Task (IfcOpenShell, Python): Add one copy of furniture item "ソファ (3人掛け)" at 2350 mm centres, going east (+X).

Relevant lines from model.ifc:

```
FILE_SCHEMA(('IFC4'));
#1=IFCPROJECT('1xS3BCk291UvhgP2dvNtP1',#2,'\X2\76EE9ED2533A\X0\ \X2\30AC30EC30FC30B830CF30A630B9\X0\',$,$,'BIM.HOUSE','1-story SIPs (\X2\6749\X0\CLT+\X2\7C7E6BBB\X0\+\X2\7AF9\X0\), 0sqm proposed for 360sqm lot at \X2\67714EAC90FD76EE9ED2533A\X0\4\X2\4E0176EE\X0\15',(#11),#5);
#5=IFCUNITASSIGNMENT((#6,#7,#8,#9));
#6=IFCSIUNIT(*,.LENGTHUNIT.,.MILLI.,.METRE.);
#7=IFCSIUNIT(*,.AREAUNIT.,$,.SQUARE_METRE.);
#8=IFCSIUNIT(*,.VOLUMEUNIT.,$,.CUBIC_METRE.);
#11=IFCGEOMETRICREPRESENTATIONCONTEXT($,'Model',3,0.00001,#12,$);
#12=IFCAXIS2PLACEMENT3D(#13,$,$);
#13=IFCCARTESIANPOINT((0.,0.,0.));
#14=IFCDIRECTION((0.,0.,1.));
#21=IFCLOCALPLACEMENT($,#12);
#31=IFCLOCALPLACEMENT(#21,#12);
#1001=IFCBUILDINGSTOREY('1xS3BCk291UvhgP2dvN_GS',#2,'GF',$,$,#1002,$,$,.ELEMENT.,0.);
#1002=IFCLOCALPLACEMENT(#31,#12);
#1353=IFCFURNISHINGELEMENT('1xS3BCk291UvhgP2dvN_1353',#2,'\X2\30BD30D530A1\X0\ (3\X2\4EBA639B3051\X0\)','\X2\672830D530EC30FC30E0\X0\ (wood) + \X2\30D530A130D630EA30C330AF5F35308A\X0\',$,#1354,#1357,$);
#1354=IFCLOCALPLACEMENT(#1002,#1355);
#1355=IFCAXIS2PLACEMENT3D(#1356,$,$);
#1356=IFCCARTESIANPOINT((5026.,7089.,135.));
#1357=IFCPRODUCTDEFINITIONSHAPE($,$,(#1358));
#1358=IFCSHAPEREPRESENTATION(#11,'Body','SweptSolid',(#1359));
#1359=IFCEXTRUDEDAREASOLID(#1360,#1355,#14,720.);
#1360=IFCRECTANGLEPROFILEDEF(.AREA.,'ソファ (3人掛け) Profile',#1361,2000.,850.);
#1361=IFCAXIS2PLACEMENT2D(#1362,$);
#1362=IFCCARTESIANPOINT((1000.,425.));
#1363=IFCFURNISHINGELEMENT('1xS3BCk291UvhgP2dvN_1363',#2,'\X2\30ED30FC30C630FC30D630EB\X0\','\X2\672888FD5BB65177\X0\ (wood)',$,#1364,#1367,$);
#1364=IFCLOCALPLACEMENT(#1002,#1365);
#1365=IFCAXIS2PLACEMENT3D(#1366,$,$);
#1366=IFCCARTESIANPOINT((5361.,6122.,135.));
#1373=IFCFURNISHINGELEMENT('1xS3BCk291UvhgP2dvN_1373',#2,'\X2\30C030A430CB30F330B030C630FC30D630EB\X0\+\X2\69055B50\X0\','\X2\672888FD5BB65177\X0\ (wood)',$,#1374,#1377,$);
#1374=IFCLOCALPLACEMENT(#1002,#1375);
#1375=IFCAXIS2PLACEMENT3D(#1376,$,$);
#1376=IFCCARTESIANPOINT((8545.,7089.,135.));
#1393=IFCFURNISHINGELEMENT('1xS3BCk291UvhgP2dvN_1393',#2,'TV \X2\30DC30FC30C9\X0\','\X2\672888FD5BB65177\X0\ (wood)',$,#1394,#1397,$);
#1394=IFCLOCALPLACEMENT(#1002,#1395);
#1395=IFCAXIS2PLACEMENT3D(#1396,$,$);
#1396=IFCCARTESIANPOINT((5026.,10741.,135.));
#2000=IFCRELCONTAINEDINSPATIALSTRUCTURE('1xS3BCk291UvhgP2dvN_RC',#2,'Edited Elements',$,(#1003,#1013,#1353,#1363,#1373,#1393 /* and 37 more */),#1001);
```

```python
import numpy as np
import ifcopenshell
import ifcopenshell.api.geometry
import ifcopenshell.api.root
import ifcopenshell.util.element
import ifcopenshell.util.placement
import ifcopenshell.util.unit

model = ifcopenshell.open("model.ifc")
unit_scale = ifcopenshell.util.unit.calculate_unit_scale(model)


def reuse_history(source, copy):
    """copy_class also copies each property set's owner history, people and application; keep the originals."""
    for rel in copy.IsDefinedBy:
        if rel.is_a("IfcRelDefinesByProperties") and (history := rel.RelatingPropertyDefinition.OwnerHistory):
            rel.RelatingPropertyDefinition.OwnerHistory = source.OwnerHistory
            ifcopenshell.util.element.remove_deep2(model, history)


source = model.by_guid("1xS3BCk291UvhgP2dvN_1353")
base = ifcopenshell.util.placement.get_local_placement(source.ObjectPlacement)
step = np.array([1.0, 0.0, 0.0]) * 2.35 / unit_scale

for i in range(1, 2):
    copy = ifcopenshell.api.root.copy_class(model, product=source)
    copy.Representation = ifcopenshell.util.element.copy_deep(
        model, source.Representation, exclude=["IfcGeometricRepresentationContext", "IfcRepresentationMap"]
    )
    reuse_history(source, copy)
    matrix = base.copy()
    matrix[:3, 3] += i * step
    print("added at", matrix[:3, 3].round(3) + 0.0)
    ifcopenshell.api.geometry.edit_object_placement(model, product=copy, matrix=matrix, is_si=False)

model.write("model_rev.ifc")
```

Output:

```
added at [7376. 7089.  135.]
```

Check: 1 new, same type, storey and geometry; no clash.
